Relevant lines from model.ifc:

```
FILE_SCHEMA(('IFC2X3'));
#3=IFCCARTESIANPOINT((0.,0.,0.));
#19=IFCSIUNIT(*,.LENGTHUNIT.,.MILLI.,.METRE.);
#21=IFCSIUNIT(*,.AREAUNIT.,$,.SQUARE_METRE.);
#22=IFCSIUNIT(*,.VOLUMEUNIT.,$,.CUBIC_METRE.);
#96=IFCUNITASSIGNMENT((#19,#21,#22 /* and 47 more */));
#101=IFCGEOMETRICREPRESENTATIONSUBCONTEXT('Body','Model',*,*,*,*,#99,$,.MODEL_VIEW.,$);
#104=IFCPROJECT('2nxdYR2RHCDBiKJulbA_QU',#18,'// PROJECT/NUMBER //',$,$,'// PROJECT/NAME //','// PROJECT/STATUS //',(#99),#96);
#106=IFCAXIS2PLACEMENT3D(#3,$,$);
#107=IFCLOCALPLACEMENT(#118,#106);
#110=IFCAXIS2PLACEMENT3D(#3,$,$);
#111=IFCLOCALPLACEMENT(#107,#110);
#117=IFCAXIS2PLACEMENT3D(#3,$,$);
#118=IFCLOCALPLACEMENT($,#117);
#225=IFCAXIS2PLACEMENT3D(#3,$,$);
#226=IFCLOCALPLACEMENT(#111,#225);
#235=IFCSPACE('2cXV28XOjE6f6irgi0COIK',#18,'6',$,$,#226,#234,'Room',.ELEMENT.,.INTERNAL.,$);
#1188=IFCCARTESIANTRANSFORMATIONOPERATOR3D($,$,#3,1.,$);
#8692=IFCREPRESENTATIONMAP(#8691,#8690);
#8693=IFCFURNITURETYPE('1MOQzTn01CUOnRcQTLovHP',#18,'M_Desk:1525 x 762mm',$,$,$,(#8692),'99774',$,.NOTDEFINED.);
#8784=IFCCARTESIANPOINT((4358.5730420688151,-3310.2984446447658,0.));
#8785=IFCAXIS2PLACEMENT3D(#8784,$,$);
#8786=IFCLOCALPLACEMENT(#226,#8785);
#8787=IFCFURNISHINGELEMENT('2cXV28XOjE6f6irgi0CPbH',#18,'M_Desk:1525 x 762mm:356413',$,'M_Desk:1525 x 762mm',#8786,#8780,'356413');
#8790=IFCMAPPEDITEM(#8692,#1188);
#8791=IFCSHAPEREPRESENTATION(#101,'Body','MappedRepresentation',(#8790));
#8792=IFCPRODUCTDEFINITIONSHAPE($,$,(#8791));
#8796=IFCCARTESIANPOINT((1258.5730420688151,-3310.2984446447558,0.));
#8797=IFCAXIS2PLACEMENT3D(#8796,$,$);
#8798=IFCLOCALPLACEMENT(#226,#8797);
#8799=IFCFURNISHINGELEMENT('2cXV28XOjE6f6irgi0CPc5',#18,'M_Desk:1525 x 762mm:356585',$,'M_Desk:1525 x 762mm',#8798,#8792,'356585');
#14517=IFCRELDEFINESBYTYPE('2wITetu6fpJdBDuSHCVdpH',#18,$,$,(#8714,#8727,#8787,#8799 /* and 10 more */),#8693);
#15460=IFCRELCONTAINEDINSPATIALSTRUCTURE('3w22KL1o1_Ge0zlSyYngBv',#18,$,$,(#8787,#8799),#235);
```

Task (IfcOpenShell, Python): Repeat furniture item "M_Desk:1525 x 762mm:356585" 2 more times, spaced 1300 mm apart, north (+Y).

```python
import numpy as np
import ifcopenshell
import ifcopenshell.api.geometry
import ifcopenshell.api.root
import ifcopenshell.util.element
import ifcopenshell.util.placement
import ifcopenshell.util.unit

model = ifcopenshell.open("model.ifc")
unit_scale = ifcopenshell.util.unit.calculate_unit_scale(model)


def reuse_history(source, copy):
    """copy_class also copies each property set's owner history, people and application; keep the originals."""
    for rel in copy.IsDefinedBy:
        if rel.is_a("IfcRelDefinesByProperties") and (history := rel.RelatingPropertyDefinition.OwnerHistory):
            rel.RelatingPropertyDefinition.OwnerHistory = source.OwnerHistory
            ifcopenshell.util.element.remove_deep2(model, history)


source = model.by_guid("2cXV28XOjE6f6irgi0CPc5")
base = ifcopenshell.util.placement.get_local_placement(source.ObjectPlacement)
step = np.array([0.0, 1.0, 0.0]) * 1.3 / unit_scale

for i in range(1, 3):
    copy = ifcopenshell.api.root.copy_class(model, product=source)
    copy.Representation = ifcopenshell.util.element.copy_deep(
        model, source.Representation, exclude=["IfcGeometricRepresentationContext", "IfcRepresentationMap"]
    )
    copy.Name = "M_Desk:1525 x 762mm"
    copy.Tag = None
    reuse_history(source, copy)
    matrix = base.copy()
    matrix[:3, 3] += i * step
    print("added at", matrix[:3, 3].round(3) + 0.0)
    ifcopenshell.api.geometry.edit_object_placement(model, product=copy, matrix=matrix, is_si=False)

model.write("model-out.ifc")
```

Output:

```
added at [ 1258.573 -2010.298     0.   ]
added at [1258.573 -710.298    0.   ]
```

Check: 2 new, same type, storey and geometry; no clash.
